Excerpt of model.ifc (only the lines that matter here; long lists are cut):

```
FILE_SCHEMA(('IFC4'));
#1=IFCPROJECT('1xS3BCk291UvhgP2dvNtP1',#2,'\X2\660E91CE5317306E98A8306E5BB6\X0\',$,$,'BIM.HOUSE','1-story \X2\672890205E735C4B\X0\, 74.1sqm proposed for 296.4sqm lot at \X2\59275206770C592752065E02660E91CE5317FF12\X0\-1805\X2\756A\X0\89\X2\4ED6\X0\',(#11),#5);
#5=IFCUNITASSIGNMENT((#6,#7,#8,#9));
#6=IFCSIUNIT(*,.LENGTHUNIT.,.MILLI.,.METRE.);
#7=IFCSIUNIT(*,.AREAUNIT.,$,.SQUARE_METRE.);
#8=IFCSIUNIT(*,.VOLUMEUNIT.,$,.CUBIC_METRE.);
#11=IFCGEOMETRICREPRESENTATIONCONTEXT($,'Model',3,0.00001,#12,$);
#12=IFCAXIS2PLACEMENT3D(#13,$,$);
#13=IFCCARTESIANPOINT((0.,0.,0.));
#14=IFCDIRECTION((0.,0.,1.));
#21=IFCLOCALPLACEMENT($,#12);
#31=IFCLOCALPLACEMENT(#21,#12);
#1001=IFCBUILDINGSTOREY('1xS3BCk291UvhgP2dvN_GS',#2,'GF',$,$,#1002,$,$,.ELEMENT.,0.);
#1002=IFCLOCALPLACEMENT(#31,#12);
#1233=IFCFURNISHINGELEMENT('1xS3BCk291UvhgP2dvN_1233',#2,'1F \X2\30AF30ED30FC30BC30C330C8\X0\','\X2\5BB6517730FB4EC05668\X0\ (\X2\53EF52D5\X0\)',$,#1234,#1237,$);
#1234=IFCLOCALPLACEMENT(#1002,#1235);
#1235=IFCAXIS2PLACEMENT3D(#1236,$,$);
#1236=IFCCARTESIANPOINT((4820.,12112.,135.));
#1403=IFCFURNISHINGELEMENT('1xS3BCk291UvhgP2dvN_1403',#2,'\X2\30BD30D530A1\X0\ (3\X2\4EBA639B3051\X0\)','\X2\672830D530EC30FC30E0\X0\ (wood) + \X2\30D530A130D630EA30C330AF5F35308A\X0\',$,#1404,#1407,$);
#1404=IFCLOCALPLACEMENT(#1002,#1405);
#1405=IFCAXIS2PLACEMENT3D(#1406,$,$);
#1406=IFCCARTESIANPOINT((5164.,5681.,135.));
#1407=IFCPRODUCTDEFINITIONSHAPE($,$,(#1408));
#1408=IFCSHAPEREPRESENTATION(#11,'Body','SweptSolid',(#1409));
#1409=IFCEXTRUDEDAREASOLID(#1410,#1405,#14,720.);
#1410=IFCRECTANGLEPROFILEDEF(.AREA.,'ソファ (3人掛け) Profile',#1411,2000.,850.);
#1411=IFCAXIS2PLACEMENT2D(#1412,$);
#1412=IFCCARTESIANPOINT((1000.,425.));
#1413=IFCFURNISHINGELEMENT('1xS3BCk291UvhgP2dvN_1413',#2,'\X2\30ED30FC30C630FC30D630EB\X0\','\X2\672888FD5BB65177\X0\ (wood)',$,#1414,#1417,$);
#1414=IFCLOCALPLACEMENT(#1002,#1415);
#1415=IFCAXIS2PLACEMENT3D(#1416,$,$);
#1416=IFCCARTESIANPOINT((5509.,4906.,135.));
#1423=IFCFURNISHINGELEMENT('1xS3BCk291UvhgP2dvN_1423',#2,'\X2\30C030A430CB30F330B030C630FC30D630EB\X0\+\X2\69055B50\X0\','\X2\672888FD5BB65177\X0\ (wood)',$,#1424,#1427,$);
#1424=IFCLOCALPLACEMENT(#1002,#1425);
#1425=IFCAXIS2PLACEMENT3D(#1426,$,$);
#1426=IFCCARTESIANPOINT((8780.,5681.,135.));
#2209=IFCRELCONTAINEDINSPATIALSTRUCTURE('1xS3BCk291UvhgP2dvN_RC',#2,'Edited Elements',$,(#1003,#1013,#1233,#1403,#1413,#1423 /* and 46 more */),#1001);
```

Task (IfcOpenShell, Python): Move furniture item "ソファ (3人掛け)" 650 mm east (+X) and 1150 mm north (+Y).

```python
import ifcopenshell
import ifcopenshell.api.geometry
import ifcopenshell.util.placement

model = ifcopenshell.open("model.ifc")

item = model.by_guid("1xS3BCk291UvhgP2dvN_1403")
matrix = ifcopenshell.util.placement.get_local_placement(item.ObjectPlacement)
matrix[0, 3] += 650.0
matrix[1, 3] += 1150.0
ifcopenshell.api.geometry.edit_object_placement(model, product=item, matrix=matrix, is_si=False)

print(ifcopenshell.util.placement.get_local_placement(item.ObjectPlacement).round(3) + 0.0)

model.write("model_rev.ifc")
```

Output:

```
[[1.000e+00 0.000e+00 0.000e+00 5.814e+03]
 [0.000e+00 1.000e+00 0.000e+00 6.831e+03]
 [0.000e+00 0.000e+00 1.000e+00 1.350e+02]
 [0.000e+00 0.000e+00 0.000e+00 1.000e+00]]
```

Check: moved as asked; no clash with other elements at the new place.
